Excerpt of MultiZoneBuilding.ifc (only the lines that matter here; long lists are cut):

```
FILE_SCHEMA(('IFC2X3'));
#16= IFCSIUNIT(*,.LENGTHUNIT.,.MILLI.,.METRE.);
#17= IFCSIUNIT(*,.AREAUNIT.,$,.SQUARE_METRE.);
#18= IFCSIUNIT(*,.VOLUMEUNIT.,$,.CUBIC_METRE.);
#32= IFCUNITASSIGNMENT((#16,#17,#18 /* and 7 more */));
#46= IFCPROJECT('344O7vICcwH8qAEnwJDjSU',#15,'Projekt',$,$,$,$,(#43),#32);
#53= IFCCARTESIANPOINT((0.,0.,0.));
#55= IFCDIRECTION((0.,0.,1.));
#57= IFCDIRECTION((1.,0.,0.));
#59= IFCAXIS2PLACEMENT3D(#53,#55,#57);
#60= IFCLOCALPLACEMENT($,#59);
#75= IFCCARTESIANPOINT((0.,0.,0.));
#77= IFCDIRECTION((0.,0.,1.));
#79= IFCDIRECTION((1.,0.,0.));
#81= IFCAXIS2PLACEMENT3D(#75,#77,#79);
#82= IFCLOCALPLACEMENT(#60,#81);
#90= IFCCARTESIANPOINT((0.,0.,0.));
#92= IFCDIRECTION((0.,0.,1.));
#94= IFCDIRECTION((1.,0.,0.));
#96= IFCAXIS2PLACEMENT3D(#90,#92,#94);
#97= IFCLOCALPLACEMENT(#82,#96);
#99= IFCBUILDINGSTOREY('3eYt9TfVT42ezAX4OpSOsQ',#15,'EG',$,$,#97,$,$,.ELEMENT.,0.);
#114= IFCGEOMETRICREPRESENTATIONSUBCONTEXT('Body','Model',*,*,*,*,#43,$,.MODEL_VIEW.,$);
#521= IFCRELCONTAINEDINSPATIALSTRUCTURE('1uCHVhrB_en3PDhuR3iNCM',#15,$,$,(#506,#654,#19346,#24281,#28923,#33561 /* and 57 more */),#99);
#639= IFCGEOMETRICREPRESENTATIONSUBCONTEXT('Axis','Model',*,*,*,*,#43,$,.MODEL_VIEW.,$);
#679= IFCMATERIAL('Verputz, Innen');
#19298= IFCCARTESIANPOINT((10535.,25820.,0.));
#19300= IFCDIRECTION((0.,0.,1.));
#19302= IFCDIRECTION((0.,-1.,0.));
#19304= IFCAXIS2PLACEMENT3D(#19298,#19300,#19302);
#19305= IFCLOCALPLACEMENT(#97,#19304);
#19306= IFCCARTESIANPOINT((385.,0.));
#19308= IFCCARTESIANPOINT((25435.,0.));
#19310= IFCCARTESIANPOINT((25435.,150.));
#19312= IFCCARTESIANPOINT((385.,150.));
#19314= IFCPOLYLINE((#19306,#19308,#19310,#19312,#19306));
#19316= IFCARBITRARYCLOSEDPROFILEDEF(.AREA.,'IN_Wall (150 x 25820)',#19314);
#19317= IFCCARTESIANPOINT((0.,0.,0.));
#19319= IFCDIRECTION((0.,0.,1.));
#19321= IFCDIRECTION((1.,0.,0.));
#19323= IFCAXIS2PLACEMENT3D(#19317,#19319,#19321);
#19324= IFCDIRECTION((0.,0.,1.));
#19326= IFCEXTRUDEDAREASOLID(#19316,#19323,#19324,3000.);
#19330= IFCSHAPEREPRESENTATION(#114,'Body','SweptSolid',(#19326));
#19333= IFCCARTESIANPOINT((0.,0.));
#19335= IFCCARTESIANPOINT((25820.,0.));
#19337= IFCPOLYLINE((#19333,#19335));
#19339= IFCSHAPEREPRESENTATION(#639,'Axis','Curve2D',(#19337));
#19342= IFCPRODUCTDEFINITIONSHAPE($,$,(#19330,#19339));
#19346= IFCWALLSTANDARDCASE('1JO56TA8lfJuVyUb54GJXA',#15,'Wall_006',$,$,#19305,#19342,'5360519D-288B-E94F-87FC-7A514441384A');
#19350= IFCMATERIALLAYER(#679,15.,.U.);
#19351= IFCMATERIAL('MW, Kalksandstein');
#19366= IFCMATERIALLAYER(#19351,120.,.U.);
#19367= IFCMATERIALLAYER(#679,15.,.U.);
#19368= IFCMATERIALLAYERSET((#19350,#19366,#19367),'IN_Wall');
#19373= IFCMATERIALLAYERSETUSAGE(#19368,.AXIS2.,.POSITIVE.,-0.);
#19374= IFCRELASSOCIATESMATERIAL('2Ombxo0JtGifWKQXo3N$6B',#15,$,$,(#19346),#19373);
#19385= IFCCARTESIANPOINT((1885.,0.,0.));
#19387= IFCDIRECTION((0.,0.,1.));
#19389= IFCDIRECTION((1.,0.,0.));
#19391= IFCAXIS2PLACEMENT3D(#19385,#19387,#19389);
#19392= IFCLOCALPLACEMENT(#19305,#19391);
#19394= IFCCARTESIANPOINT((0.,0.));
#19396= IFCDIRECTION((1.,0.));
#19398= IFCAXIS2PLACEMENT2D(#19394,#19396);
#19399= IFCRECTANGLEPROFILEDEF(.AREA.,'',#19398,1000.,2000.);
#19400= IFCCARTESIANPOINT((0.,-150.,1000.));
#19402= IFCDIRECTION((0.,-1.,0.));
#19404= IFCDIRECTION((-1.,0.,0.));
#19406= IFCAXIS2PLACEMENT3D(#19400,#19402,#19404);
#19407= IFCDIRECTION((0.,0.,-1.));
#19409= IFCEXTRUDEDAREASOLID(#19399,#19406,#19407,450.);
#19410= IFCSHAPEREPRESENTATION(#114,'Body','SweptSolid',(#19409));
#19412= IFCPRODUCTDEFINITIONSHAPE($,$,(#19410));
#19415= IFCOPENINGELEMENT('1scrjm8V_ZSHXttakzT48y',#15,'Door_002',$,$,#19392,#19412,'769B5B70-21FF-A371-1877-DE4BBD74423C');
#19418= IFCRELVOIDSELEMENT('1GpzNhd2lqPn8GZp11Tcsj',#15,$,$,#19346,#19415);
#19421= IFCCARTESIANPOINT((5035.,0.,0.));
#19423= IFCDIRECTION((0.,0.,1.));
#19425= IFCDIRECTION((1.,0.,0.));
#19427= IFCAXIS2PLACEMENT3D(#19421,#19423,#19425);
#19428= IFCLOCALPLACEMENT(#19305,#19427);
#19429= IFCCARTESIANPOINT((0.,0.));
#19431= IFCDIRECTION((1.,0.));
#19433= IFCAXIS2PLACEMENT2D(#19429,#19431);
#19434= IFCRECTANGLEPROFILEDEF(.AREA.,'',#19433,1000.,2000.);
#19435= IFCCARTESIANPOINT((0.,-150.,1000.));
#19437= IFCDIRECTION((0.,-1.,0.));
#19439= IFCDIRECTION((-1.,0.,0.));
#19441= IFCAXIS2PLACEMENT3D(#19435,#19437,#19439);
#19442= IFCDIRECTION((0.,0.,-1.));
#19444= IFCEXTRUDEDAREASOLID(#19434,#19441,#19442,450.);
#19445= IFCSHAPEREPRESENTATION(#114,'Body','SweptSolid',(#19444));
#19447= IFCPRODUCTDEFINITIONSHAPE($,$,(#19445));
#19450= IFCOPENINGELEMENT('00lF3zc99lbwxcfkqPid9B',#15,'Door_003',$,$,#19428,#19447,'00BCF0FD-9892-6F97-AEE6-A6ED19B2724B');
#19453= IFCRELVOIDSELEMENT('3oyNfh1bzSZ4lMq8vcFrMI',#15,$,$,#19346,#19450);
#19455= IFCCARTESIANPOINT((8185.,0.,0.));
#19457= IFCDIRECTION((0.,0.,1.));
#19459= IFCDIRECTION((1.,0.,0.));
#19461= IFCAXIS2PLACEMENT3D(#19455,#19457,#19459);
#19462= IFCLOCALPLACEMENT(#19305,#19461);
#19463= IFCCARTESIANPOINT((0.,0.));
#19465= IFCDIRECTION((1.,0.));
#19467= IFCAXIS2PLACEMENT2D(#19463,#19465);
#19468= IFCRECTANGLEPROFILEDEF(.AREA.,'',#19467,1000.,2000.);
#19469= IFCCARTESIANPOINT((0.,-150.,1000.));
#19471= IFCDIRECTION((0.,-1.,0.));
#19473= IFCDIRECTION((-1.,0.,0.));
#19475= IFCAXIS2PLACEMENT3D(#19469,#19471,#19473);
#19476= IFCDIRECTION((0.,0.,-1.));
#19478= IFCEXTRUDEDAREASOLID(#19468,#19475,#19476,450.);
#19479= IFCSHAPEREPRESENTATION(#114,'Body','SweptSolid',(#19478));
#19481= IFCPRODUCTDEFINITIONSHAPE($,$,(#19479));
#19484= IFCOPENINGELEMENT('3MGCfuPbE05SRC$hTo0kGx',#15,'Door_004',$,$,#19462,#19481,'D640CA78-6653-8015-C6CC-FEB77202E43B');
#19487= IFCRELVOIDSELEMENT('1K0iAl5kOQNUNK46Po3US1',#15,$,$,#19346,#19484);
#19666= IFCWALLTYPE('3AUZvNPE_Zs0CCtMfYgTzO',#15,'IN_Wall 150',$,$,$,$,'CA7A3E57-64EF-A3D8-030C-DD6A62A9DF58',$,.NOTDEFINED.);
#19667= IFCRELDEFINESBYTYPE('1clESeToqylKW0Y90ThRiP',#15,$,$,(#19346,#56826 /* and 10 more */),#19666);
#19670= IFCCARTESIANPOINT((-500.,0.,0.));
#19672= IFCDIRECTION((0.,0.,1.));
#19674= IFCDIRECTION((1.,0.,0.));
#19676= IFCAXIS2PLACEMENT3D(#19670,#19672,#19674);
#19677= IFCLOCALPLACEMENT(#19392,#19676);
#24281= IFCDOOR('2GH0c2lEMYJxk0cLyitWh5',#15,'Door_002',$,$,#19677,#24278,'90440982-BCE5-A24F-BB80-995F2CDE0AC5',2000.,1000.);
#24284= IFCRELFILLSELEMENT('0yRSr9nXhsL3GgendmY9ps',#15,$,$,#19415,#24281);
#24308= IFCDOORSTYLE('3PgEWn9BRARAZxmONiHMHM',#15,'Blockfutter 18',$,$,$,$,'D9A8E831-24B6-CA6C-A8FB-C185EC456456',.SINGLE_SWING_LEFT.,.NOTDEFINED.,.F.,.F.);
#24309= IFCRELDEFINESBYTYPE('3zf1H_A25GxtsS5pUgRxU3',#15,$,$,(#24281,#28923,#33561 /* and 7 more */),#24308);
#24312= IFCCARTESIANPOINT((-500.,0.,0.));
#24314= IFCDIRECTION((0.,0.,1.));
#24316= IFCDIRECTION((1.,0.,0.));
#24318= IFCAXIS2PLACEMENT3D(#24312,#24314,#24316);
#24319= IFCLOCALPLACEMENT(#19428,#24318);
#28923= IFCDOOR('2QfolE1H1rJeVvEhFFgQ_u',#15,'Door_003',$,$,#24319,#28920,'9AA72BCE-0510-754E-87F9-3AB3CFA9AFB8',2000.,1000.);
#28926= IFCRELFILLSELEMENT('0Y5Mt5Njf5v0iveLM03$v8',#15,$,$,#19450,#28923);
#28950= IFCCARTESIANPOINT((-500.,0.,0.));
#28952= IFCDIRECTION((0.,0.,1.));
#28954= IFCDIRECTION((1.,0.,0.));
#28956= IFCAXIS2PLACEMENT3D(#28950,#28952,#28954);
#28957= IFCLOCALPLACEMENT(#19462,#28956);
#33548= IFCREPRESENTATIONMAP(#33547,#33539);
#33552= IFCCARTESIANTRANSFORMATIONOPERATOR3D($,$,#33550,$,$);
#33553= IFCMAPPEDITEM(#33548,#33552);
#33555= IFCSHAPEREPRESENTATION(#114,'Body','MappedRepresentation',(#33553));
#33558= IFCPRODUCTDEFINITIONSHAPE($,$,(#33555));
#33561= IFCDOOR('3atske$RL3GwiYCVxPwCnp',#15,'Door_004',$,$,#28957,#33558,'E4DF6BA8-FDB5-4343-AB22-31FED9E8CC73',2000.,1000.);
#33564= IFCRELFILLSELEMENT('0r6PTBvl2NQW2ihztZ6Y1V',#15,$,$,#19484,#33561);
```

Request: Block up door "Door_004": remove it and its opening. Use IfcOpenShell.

```python
import ifcopenshell
import ifcopenshell.api.feature
import ifcopenshell.api.root
import ifcopenshell.geom
import ifcopenshell.util.shape

model = ifcopenshell.open("MultiZoneBuilding.ifc")
settings = ifcopenshell.geom.settings()


def volume(element):
    """Net volume in cubic metres, openings subtracted."""
    shape = ifcopenshell.geom.create_shape(settings, element)
    return ifcopenshell.util.shape.get_volume(shape.geometry)


door = model.by_guid("3atske$RL3GwiYCVxPwCnp")
opening = door.FillsVoids[0].RelatingOpeningElement
wall = opening.VoidsElements[0].RelatingBuildingElement
before = volume(wall)

ifcopenshell.api.root.remove_product(model, product=door)
ifcopenshell.api.feature.remove_feature(model, feature=opening)

after = volume(wall)

print(f"wall volume {before:.3f} -> {after:.3f} m3")

model.write("MultiZoneBuilding_rev.ifc")
```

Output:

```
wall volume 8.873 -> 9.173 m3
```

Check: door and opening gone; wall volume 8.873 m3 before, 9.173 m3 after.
